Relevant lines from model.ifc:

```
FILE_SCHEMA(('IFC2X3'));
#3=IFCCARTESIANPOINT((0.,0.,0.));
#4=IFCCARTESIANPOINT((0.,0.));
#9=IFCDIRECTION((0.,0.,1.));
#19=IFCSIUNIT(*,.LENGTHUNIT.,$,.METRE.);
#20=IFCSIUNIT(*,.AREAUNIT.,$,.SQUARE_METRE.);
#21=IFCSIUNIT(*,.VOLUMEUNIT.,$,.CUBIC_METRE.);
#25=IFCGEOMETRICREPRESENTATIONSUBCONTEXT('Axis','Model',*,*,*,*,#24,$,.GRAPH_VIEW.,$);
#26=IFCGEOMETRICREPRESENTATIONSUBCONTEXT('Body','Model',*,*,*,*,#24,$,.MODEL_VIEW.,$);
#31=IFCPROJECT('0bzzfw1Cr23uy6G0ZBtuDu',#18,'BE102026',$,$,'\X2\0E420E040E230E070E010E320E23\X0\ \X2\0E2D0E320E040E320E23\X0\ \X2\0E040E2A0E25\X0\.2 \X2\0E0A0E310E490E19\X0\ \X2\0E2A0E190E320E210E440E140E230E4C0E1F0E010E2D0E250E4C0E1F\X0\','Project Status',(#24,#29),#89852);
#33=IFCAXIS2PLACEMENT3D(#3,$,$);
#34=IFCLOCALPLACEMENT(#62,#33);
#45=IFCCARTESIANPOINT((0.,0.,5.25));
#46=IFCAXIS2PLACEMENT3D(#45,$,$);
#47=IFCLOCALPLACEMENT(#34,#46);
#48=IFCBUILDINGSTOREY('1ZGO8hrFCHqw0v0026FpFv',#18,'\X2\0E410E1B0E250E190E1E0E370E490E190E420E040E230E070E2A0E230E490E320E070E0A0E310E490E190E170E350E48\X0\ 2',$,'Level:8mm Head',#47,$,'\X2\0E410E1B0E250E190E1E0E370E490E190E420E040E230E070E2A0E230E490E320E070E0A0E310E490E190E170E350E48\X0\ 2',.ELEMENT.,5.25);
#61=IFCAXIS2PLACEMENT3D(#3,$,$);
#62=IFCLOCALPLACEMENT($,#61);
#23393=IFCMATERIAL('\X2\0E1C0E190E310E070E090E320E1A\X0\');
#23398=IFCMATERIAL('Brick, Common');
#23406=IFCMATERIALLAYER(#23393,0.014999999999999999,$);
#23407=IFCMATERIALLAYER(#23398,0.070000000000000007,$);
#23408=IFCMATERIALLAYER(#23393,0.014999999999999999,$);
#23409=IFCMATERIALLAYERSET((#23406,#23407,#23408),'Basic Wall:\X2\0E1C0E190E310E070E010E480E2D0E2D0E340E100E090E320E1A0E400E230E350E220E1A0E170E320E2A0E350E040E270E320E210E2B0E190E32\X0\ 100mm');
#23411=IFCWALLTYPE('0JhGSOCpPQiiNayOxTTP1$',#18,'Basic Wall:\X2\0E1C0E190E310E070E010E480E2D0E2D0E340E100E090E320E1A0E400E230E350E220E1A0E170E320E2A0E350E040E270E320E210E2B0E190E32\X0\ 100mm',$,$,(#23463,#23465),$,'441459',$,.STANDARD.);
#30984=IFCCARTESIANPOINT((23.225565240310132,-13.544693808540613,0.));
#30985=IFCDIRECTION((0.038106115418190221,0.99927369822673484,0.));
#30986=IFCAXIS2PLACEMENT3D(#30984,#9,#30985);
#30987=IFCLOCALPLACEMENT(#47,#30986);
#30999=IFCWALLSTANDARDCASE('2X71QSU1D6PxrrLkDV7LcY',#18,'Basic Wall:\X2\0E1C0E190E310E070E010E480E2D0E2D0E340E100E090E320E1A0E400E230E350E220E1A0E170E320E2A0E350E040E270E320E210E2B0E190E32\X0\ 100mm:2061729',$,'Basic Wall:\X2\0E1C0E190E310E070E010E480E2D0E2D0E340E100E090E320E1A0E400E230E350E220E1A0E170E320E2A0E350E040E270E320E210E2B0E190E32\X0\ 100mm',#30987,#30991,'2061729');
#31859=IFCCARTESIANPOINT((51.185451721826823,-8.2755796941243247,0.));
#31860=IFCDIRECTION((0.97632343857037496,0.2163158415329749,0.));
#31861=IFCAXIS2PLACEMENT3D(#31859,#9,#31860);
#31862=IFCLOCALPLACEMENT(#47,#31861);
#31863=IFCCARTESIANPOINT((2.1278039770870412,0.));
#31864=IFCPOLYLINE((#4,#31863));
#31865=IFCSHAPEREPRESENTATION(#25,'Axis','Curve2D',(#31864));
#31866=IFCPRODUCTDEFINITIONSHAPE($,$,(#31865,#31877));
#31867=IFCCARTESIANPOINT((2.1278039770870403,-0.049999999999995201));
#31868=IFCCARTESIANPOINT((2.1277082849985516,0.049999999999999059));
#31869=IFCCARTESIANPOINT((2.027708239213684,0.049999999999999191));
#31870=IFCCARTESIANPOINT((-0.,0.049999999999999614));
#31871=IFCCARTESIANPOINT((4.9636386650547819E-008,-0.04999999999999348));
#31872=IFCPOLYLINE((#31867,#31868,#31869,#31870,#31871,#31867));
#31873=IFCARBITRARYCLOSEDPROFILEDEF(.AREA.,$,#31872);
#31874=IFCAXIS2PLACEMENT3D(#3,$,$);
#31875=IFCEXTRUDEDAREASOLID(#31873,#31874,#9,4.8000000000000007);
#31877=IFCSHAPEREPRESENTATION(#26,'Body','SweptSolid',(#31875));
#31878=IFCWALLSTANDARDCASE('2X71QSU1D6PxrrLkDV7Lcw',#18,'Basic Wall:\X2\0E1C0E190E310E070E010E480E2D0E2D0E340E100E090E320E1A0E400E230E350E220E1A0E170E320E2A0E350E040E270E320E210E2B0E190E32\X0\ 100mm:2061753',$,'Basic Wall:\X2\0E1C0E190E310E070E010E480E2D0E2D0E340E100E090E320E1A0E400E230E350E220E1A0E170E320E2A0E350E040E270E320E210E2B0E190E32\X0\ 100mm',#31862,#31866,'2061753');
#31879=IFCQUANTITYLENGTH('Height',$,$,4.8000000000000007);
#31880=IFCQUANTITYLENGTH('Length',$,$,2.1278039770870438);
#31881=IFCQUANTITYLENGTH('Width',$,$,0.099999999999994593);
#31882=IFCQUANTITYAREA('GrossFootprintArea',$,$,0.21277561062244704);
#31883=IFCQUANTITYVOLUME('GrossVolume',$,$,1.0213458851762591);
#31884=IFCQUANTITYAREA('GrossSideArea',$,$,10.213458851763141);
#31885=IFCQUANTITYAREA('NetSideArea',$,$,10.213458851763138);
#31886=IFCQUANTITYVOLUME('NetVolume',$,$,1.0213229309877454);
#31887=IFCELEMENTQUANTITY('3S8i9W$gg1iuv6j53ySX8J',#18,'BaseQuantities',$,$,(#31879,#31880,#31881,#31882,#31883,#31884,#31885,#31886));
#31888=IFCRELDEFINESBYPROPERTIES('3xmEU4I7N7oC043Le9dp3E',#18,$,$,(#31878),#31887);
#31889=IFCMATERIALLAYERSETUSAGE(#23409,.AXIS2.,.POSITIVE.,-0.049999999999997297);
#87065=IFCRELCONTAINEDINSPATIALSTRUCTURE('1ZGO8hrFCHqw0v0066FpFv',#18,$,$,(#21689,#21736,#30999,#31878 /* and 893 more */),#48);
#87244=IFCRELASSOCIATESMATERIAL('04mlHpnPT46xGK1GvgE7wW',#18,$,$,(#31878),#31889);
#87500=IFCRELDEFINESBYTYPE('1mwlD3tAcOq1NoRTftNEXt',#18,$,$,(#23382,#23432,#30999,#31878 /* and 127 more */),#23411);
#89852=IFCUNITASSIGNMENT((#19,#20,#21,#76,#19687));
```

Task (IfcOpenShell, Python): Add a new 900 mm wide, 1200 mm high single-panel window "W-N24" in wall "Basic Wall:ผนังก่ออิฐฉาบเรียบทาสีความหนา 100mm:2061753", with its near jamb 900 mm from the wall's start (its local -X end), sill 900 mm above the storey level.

```python
import numpy as np
import ifcopenshell
import ifcopenshell.api.feature
import ifcopenshell.api.geometry
import ifcopenshell.api.pset
import ifcopenshell.api.root
import ifcopenshell.api.spatial
import ifcopenshell.api.type
import ifcopenshell.geom
import ifcopenshell.util.element
import ifcopenshell.util.placement
import ifcopenshell.util.representation
import ifcopenshell.util.shape
import ifcopenshell.util.unit

model = ifcopenshell.open("model.ifc")
unit_scale = ifcopenshell.util.unit.calculate_unit_scale(model)
area_scale = ifcopenshell.util.unit.calculate_unit_scale(model, "AREAUNIT")
volume_scale = ifcopenshell.util.unit.calculate_unit_scale(model, "VOLUMEUNIT")
settings = ifcopenshell.geom.settings()


def volume(element):
    """Net volume in cubic metres, openings subtracted."""
    shape = ifcopenshell.geom.create_shape(settings, element)
    return ifcopenshell.util.shape.get_volume(shape.geometry)


wall = model.by_id(31878)
storey = ifcopenshell.util.element.get_container(wall, ifc_class="IfcBuildingStorey")
context = ifcopenshell.util.representation.get_context(model, "Model", "Body", "MODEL_VIEW")
before = volume(wall)

width, height, from_end, sill = 0.9, 1.2, 0.9, 0.9  # metres

# The wall runs along its own X axis, and the end named is its -X end.
wall_shape = ifcopenshell.geom.create_shape(settings, wall)
x, y, z = ifcopenshell.util.shape.get_vertices(wall_shape.geometry).T
start = x.min() + from_end
face, thickness = float(y.min()), float(y.max() - y.min())
wall_matrix = ifcopenshell.util.placement.get_local_placement(wall.ObjectPlacement)
level = ifcopenshell.util.placement.get_local_placement(storey.ObjectPlacement)[2, 3]


def in_wall(x, y):
    """Placement at x, y metres in the wall's axes, at sill height."""
    matrix = wall_matrix.copy()
    matrix[:, 3] = wall_matrix @ np.array([x / unit_scale, y / unit_scale, 0.0, 1.0])
    matrix[2, 3] = level + sill / unit_scale
    return matrix


# Opening: a box that overshoots both wall faces by 50 mm.
opening = ifcopenshell.api.root.create_entity(model, ifc_class="IfcOpeningElement")
box = ifcopenshell.api.geometry.add_wall_representation(
    model, context=context, length=width, height=height, thickness=thickness + 0.1
)
ifcopenshell.api.geometry.assign_representation(model, product=opening, representation=box)
ifcopenshell.api.geometry.edit_object_placement(model, product=opening, matrix=in_wall(start, face - 0.05), is_si=False)
ifcopenshell.api.feature.add_feature(model, feature=opening, element=wall)

window = ifcopenshell.api.root.create_entity(model, ifc_class="IfcWindow", name="W-N24")
window.OverallWidth, window.OverallHeight = width / unit_scale, height / unit_scale
body = ifcopenshell.api.geometry.add_window_representation(
    model,
    context=context,
    overall_width=window.OverallWidth,
    overall_height=window.OverallHeight,
    partition_type="SINGLE_PANEL",
)
ifcopenshell.api.geometry.assign_representation(model, product=window, representation=body)
ifcopenshell.api.spatial.assign_container(model, products=[window], relating_structure=storey)
fills = ifcopenshell.api.feature.add_filling(model, opening=opening, element=window)
fills.OwnerHistory = window.OwnerHistory  # required in IFC2X3

# IFC2X3 keeps the operation on the window style.
style = ifcopenshell.api.root.create_entity(model, ifc_class="IfcWindowStyle", name="W-N24")
style.OperationType, style.ConstructionType = "SINGLE_PANEL", "NOTDEFINED"
style.ParameterTakesPrecedence = style.Sizeable = False
ifcopenshell.api.type.assign_type(model, related_objects=[window], relating_type=style)

# Centre the window in the wall's thickness.
ifcopenshell.api.geometry.edit_object_placement(model, product=window, matrix=in_wall(start, face), is_si=False)
window_shape = ifcopenshell.geom.create_shape(settings, window)
depth = ifcopenshell.util.shape.get_vertices(window_shape.geometry)[:, 1]
offset = face + thickness / 2 - (depth.min() + depth.max()) / 2
ifcopenshell.api.geometry.edit_object_placement(model, product=window, matrix=in_wall(start, offset), is_si=False)

after = volume(wall)

# Update the wall's stored quantities.
qto = model.by_id(ifcopenshell.util.element.get_pset(wall, "BaseQuantities", should_inherit=False)["id"])
ifcopenshell.api.pset.edit_qto(model, qto=qto, properties={
    "NetSideArea": after / thickness / area_scale,
    "NetVolume": after / volume_scale,
})

print(f"wall volume {before:.3f} -> {after:.3f} m3")

model.write("model_updated.ifc")
```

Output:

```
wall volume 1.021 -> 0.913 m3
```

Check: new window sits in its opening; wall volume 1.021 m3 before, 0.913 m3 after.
